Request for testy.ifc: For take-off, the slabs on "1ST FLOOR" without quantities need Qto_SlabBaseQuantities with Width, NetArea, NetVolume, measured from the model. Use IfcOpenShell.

First a look at what the model holds.

```python
import ifcopenshell
import ifcopenshell.util.element
import ifcopenshell.util.unit

model = ifcopenshell.open("testy.ifc")
print(model.schema)
for unit_type in ("LENGTHUNIT", "AREAUNIT", "VOLUMEUNIT"):
    print(unit_type, ifcopenshell.util.unit.calculate_unit_scale(model, unit_type))
storey = next(s for s in model.by_type("IfcBuildingStorey") if s.Name == "1ST FLOOR")
slabs = [e for e in ifcopenshell.util.element.get_decomposition(storey) if e.is_a("IfcSlab")]
for e in sorted(slabs, key=lambda e: e.id()):
    print(e.id(), e.is_a(), e.Name, list(ifcopenshell.util.element.get_psets(e, qtos_only=True)), sep=" | ")
```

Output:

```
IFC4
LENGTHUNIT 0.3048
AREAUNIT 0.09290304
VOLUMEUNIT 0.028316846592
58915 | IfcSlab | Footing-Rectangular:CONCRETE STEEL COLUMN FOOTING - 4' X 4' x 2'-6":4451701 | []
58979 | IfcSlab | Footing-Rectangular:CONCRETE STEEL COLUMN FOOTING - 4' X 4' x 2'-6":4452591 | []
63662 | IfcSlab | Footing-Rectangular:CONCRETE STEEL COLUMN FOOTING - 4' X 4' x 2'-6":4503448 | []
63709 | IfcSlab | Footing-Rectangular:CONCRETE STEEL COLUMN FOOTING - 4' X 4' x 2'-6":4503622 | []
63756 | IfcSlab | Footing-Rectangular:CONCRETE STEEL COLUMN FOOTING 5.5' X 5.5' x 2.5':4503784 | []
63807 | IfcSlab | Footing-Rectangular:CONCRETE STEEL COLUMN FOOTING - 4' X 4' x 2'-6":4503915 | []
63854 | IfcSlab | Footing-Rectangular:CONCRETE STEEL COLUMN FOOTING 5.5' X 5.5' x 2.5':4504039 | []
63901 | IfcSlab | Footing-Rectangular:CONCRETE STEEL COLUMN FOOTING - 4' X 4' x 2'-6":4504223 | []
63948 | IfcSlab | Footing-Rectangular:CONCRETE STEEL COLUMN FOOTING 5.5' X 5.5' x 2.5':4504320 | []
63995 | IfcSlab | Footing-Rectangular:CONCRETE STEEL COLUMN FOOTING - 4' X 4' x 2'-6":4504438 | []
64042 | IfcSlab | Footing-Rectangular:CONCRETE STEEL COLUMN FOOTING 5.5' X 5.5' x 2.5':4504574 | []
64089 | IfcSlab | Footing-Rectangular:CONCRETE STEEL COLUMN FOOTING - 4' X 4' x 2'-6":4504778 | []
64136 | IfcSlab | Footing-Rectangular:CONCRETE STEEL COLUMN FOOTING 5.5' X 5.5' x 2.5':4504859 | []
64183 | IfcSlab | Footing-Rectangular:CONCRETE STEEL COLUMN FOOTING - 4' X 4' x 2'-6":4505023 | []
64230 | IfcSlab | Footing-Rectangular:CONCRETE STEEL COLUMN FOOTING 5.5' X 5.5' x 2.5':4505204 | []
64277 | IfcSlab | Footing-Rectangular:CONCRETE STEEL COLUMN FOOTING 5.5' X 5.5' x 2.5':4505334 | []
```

```python
import ifcopenshell
import ifcopenshell.api.pset
import ifcopenshell.geom
import ifcopenshell.util.element
import ifcopenshell.util.shape
import ifcopenshell.util.unit

model = ifcopenshell.open("testy.ifc")
unit_scale = ifcopenshell.util.unit.calculate_unit_scale(model)
area_scale = ifcopenshell.util.unit.calculate_unit_scale(model, "AREAUNIT")
volume_scale = ifcopenshell.util.unit.calculate_unit_scale(model, "VOLUMEUNIT")
settings = ifcopenshell.geom.settings()

storey = next(s for s in model.by_type("IfcBuildingStorey") if s.Name == "1ST FLOOR")
slabs = [e for e in ifcopenshell.util.element.get_decomposition(storey) if e.is_a("IfcSlab")]

for e in sorted(slabs, key=lambda e: e.id()):
    if ifcopenshell.util.element.get_psets(e, qtos_only=True, should_inherit=False):
        continue
    # Geometry comes back in metres, in the element's own axes.
    shape = ifcopenshell.geom.create_shape(settings, e)
    values = {
        "Width": ifcopenshell.util.shape.get_z(shape.geometry) / unit_scale,
        "NetArea": ifcopenshell.util.shape.get_footprint_area(shape.geometry) / area_scale,
        "NetVolume": ifcopenshell.util.shape.get_volume(shape.geometry) / volume_scale,
    }
    qto = ifcopenshell.api.pset.add_qto(model, product=e, name="Qto_SlabBaseQuantities")
    ifcopenshell.api.pset.edit_qto(model, qto=qto, properties=values)
    print(e.id(), {k: round(v, 3) for k, v in values.items()})

model.write("testy_rev.ifc")
```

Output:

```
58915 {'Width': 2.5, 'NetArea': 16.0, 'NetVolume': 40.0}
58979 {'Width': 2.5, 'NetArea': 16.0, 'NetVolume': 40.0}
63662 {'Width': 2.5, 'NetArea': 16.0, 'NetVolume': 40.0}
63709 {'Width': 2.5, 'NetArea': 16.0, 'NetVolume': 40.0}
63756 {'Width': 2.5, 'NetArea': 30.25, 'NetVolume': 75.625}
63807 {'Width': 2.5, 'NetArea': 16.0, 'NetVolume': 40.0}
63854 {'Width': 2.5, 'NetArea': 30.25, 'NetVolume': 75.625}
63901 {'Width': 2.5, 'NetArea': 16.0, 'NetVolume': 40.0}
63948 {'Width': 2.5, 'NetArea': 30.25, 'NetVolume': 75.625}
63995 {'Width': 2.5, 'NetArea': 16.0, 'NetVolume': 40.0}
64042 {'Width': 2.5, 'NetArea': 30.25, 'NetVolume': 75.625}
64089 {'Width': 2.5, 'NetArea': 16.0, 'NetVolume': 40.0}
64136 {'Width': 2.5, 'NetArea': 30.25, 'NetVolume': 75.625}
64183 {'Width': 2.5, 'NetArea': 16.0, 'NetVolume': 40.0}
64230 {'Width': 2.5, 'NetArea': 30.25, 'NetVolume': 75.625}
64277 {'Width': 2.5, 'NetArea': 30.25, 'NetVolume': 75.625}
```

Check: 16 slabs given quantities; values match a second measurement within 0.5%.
